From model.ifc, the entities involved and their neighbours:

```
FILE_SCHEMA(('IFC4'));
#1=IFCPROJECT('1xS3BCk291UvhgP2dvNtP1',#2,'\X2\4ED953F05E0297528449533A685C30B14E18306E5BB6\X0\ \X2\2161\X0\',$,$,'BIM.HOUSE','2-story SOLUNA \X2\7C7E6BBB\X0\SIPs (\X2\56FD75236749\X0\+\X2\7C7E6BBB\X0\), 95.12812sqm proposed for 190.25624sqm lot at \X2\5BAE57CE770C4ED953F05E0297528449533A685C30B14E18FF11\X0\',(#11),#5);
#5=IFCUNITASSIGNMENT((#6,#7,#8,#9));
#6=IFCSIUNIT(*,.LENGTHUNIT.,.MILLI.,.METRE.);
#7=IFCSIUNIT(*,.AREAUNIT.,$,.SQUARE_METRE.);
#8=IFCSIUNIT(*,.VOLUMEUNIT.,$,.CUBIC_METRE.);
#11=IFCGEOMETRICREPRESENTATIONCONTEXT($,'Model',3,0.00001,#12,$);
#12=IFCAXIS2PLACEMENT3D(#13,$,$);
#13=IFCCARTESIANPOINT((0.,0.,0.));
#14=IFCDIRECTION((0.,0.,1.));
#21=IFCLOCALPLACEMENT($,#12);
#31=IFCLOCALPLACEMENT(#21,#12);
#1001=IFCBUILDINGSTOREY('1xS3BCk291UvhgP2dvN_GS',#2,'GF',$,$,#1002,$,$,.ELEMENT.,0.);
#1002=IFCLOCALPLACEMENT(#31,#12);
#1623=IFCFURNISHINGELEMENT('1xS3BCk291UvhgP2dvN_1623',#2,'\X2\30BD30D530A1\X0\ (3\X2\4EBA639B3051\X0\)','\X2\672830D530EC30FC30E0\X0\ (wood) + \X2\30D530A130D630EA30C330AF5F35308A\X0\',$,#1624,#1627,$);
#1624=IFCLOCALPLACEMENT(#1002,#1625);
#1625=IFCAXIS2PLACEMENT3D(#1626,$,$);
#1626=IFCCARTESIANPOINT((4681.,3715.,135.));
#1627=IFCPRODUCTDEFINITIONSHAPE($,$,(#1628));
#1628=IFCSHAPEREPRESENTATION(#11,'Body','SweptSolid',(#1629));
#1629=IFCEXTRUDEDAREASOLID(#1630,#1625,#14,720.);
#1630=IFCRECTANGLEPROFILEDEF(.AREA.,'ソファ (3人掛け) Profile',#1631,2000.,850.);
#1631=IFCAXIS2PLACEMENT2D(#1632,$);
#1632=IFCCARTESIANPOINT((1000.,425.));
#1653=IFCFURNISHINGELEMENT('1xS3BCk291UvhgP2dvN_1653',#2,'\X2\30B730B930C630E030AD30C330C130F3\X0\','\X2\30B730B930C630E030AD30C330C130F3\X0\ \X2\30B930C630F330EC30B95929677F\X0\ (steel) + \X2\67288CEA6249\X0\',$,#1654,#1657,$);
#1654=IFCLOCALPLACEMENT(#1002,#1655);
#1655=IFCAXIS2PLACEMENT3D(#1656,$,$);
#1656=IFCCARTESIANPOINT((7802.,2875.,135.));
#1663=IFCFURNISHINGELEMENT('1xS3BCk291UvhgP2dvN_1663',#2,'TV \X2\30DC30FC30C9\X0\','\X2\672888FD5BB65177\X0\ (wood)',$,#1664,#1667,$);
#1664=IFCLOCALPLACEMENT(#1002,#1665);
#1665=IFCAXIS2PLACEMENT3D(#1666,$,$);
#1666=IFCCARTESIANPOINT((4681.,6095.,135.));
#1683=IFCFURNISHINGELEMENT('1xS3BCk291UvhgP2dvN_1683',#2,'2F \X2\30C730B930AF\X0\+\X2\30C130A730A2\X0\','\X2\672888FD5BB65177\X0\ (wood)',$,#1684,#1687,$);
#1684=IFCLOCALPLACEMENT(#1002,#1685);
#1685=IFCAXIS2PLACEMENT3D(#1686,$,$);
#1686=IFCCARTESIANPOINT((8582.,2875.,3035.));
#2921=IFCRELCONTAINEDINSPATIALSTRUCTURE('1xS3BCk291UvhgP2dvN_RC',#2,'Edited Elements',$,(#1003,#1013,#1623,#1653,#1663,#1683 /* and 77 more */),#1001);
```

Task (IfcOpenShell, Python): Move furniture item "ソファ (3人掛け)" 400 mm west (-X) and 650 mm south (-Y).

```python
import ifcopenshell
import ifcopenshell.api.geometry
import ifcopenshell.util.placement

model = ifcopenshell.open("model.ifc")

item = model.by_guid("1xS3BCk291UvhgP2dvN_1623")
matrix = ifcopenshell.util.placement.get_local_placement(item.ObjectPlacement)
matrix[0, 3] -= 400.0
matrix[1, 3] -= 650.0
ifcopenshell.api.geometry.edit_object_placement(model, product=item, matrix=matrix, is_si=False)

print(ifcopenshell.util.placement.get_local_placement(item.ObjectPlacement).round(3) + 0.0)

model.write("model_updated.ifc")
```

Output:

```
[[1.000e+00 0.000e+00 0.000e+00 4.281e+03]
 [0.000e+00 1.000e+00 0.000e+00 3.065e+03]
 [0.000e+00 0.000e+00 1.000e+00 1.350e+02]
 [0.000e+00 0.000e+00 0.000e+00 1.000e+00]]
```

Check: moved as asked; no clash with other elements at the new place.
